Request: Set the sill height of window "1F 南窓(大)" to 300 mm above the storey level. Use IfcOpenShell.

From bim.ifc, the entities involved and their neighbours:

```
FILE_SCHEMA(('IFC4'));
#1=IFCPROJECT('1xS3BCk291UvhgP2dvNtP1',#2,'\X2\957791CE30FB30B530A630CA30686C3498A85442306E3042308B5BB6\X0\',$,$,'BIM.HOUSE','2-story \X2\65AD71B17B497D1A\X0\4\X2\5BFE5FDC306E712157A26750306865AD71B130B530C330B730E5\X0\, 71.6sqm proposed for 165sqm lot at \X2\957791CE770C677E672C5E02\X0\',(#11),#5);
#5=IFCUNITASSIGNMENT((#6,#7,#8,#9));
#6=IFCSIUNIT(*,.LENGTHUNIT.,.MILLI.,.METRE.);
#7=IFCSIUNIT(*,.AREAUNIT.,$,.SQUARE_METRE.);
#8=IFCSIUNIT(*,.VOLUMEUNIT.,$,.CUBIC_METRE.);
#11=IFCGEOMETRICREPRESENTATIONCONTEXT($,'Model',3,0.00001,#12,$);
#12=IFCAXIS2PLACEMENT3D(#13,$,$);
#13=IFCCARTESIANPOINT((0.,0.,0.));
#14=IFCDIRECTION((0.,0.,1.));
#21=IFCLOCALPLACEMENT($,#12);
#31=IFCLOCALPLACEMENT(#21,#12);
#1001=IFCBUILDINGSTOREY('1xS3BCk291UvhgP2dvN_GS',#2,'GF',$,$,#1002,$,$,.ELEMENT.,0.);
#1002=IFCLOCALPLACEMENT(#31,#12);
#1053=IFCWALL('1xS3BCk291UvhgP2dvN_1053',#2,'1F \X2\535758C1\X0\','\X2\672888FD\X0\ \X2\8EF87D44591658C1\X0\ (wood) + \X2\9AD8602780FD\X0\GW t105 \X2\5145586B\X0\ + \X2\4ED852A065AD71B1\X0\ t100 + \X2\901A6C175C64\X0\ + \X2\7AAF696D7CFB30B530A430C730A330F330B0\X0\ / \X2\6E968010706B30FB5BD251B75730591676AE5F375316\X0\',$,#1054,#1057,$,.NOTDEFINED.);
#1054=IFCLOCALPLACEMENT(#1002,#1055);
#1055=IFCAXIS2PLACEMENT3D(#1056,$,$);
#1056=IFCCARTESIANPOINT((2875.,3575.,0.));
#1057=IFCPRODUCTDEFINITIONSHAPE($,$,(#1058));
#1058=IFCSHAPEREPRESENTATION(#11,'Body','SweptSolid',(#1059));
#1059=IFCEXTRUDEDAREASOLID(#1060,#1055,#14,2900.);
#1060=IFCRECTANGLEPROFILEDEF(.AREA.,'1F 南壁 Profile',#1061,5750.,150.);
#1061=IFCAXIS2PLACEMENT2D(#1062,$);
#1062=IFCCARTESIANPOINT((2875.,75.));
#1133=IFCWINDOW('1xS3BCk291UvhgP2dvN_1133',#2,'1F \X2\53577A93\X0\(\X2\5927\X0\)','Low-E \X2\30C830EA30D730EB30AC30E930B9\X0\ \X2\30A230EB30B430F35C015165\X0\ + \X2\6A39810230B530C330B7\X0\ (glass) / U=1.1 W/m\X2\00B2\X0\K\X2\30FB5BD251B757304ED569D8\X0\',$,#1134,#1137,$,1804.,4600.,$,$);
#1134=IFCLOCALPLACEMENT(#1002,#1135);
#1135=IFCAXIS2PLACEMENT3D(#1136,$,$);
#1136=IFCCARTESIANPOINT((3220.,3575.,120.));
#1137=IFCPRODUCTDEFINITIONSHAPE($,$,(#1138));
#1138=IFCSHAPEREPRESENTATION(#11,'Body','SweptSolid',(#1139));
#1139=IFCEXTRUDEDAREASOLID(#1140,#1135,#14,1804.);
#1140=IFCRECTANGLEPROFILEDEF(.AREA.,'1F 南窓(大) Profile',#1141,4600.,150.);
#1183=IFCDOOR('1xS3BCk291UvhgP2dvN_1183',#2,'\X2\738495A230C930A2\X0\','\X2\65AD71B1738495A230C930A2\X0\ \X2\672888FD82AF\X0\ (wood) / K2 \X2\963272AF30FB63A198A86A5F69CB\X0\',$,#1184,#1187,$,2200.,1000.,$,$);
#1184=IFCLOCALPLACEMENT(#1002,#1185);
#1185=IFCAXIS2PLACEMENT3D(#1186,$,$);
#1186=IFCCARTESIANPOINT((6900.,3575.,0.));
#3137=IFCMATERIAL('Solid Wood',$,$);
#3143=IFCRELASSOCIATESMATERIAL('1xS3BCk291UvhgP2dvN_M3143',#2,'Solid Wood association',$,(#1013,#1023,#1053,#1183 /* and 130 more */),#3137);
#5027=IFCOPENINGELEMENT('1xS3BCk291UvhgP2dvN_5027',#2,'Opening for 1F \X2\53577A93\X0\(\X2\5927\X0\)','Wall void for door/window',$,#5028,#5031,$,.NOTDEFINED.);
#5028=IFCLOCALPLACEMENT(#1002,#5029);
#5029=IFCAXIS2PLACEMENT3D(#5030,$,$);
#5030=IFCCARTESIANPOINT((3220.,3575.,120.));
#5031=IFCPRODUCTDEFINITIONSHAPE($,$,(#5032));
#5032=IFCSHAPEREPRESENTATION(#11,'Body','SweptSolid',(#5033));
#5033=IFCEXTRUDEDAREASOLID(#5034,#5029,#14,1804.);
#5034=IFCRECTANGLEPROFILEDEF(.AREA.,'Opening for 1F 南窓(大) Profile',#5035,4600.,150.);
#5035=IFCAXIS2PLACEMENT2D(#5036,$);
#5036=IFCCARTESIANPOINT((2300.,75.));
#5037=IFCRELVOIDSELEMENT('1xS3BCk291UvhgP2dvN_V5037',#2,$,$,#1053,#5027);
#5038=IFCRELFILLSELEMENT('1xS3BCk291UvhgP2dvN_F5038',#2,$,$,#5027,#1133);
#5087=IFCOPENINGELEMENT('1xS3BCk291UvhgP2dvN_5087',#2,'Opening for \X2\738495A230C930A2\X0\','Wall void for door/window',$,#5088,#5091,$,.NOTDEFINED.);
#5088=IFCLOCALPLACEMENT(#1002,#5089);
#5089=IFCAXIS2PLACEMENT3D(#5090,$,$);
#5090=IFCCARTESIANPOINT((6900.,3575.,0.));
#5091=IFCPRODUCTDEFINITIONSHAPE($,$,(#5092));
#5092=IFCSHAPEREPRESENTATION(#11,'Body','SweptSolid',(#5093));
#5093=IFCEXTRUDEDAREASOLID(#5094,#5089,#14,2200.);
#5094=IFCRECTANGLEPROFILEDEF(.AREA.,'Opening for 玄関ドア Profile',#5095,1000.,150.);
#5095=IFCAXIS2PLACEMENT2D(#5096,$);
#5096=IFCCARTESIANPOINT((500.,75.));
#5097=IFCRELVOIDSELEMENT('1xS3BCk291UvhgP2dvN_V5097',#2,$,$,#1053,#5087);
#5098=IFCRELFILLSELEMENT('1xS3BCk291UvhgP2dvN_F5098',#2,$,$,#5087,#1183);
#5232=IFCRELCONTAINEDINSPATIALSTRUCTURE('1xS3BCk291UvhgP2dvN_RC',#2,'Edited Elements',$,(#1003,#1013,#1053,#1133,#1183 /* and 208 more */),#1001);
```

```python
import numpy as np
import ifcopenshell
import ifcopenshell.api.geometry
import ifcopenshell.geom
import ifcopenshell.util.element
import ifcopenshell.util.placement
import ifcopenshell.util.shape
import ifcopenshell.util.unit

model = ifcopenshell.open("bim.ifc")
unit_scale = ifcopenshell.util.unit.calculate_unit_scale(model)

window = model.by_guid("1xS3BCk291UvhgP2dvN_1133")
opening = window.FillsVoids[0].RelatingOpeningElement
storey = ifcopenshell.util.element.get_container(window, ifc_class="IfcBuildingStorey")
level = ifcopenshell.util.placement.get_local_placement(storey.ObjectPlacement)[2, 3]

# The opening's origin need not be at the sill, so measure its lowest point.
shape = ifcopenshell.geom.create_shape(ifcopenshell.geom.settings(), opening)
bottom = ifcopenshell.util.shape.get_shape_bottom_elevation(shape, shape.geometry) / unit_scale
dz = level + 0.3 / unit_scale - bottom

shift = np.array([0.0, 0.0, dz])
# The window is not placed relative to its opening, so move both.
for product in (opening, window):
    matrix = ifcopenshell.util.placement.get_local_placement(product.ObjectPlacement)
    matrix[:3, 3] += shift
    ifcopenshell.api.geometry.edit_object_placement(model, product=product, matrix=matrix, is_si=False)

print(f"moved by {dz * unit_scale:+.3f} m")

model.write("bim_edited.ifc")
```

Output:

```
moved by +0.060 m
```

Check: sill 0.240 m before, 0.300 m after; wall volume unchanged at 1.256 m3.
